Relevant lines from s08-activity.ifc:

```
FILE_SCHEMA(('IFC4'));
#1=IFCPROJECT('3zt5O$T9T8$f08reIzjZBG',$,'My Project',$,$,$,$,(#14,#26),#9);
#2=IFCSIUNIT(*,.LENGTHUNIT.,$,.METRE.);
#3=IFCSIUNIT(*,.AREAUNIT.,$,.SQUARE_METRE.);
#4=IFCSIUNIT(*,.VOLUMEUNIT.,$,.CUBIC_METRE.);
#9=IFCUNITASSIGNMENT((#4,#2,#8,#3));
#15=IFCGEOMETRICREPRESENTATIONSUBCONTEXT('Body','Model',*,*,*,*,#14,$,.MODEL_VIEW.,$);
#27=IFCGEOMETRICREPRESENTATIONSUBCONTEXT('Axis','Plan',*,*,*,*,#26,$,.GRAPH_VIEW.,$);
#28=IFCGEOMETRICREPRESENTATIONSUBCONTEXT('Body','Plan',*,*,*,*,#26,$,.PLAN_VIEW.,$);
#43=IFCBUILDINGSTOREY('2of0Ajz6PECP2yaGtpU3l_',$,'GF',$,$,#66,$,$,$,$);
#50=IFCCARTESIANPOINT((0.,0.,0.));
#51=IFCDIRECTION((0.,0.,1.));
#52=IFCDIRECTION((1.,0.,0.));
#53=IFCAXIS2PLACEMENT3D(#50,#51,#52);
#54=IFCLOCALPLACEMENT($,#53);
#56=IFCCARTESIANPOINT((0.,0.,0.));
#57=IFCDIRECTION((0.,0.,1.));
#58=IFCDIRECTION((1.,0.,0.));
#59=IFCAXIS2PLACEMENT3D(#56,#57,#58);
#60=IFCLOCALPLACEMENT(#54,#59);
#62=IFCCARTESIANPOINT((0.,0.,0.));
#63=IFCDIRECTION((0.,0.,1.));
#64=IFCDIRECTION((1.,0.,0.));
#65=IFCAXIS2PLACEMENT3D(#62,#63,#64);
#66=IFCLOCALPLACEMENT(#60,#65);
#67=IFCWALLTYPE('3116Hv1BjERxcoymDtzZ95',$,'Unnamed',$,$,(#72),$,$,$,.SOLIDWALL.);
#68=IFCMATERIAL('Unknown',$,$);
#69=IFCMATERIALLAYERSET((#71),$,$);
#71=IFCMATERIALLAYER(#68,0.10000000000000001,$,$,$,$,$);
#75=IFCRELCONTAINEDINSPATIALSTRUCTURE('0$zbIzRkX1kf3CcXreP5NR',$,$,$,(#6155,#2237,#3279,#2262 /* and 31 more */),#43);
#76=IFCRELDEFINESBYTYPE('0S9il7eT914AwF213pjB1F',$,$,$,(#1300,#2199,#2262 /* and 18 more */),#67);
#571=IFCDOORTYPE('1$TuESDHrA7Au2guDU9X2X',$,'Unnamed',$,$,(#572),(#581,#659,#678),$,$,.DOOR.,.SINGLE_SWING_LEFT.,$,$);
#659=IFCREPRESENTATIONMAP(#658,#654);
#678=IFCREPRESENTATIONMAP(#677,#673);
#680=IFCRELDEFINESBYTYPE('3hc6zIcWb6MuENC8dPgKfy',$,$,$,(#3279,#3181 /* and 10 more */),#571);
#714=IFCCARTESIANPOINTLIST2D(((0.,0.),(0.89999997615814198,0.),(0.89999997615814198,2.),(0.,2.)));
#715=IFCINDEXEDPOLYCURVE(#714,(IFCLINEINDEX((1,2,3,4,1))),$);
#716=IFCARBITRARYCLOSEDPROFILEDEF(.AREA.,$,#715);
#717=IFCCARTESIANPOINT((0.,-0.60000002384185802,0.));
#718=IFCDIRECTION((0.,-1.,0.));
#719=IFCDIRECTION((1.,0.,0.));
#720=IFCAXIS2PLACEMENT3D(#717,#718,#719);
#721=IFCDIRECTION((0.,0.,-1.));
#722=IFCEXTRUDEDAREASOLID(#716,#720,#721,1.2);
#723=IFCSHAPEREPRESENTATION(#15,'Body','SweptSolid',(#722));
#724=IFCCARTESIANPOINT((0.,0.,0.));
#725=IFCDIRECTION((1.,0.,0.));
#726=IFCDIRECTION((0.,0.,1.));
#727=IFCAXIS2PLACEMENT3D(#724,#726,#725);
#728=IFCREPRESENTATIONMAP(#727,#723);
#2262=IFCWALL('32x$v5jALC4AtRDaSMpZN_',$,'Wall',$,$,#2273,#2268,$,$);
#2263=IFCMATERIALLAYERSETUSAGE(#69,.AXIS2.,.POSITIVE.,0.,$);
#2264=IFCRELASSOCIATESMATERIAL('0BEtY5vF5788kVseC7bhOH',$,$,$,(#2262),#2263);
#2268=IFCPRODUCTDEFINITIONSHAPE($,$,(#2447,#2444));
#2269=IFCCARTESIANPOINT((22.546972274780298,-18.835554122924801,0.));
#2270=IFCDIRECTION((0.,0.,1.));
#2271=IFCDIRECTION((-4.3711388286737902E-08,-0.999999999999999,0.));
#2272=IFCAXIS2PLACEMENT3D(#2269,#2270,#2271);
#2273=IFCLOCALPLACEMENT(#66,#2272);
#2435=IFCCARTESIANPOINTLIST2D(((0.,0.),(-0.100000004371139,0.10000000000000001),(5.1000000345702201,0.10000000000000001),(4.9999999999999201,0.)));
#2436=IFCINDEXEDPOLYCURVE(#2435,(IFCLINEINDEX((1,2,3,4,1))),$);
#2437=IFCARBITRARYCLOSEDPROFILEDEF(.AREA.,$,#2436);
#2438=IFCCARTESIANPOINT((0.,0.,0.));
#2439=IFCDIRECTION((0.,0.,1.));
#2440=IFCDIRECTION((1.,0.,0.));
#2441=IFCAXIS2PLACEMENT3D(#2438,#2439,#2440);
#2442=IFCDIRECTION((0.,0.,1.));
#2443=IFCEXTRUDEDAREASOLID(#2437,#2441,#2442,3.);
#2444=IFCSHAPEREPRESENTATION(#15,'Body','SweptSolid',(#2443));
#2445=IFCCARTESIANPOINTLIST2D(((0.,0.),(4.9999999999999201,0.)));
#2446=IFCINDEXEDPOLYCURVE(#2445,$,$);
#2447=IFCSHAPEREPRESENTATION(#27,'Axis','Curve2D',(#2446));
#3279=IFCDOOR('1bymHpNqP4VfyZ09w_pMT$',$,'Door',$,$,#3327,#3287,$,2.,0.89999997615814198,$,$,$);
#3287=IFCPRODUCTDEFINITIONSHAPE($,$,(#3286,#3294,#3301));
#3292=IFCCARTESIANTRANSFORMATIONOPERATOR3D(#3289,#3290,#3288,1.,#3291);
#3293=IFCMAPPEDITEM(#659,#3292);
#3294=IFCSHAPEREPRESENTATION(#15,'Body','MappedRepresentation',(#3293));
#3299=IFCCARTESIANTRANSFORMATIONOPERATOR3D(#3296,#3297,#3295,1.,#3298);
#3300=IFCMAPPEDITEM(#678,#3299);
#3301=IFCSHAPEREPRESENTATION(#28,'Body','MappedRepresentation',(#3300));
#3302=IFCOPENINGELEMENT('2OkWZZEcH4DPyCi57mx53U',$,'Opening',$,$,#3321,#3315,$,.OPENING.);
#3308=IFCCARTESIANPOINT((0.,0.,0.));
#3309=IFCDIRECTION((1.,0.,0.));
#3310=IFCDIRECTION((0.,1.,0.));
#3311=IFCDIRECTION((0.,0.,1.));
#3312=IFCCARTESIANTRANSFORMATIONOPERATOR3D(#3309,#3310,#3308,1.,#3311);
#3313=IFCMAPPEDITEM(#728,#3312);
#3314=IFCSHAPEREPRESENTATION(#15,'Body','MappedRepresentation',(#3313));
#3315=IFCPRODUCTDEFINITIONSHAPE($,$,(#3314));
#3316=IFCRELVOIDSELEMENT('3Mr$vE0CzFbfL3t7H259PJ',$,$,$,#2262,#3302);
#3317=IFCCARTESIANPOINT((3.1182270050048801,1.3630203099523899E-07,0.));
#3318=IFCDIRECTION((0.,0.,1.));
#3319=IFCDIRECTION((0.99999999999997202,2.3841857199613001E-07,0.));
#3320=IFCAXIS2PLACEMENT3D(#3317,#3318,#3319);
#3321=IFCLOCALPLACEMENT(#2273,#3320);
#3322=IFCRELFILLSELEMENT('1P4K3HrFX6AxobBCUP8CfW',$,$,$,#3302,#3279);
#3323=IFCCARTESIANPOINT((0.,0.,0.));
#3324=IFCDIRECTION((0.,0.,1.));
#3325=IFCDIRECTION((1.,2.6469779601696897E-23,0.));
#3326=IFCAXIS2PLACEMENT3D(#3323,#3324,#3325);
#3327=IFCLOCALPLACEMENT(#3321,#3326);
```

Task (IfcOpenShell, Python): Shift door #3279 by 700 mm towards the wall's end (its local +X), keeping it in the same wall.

```python
import ifcopenshell
import ifcopenshell.api.geometry
import ifcopenshell.util.placement
import ifcopenshell.util.unit

model = ifcopenshell.open("s08-activity.ifc")
unit_scale = ifcopenshell.util.unit.calculate_unit_scale(model)

door = model.by_guid("1bymHpNqP4VfyZ09w_pMT$")
opening = door.FillsVoids[0].RelatingOpeningElement
wall = opening.VoidsElements[0].RelatingBuildingElement

wall_matrix = ifcopenshell.util.placement.get_local_placement(wall.ObjectPlacement)
shift = wall_matrix[:3, 0] * 0.7 / unit_scale
before = ifcopenshell.util.placement.get_local_placement(door.ObjectPlacement)[:3, 3].copy()

# The door is placed relative to its opening, so it follows when the opening moves.
matrix = ifcopenshell.util.placement.get_local_placement(opening.ObjectPlacement)
matrix[:3, 3] += shift
ifcopenshell.api.geometry.edit_object_placement(
    model, product=opening, matrix=matrix, is_si=False, should_transform_children=True
)

after = ifcopenshell.util.placement.get_local_placement(door.ObjectPlacement)[:3, 3]
print("door moved by", (after - before).round(3) + 0.0)

model.write("s08-activity-out.ifc")
```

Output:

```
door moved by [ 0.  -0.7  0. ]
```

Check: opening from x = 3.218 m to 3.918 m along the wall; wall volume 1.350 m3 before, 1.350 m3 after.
